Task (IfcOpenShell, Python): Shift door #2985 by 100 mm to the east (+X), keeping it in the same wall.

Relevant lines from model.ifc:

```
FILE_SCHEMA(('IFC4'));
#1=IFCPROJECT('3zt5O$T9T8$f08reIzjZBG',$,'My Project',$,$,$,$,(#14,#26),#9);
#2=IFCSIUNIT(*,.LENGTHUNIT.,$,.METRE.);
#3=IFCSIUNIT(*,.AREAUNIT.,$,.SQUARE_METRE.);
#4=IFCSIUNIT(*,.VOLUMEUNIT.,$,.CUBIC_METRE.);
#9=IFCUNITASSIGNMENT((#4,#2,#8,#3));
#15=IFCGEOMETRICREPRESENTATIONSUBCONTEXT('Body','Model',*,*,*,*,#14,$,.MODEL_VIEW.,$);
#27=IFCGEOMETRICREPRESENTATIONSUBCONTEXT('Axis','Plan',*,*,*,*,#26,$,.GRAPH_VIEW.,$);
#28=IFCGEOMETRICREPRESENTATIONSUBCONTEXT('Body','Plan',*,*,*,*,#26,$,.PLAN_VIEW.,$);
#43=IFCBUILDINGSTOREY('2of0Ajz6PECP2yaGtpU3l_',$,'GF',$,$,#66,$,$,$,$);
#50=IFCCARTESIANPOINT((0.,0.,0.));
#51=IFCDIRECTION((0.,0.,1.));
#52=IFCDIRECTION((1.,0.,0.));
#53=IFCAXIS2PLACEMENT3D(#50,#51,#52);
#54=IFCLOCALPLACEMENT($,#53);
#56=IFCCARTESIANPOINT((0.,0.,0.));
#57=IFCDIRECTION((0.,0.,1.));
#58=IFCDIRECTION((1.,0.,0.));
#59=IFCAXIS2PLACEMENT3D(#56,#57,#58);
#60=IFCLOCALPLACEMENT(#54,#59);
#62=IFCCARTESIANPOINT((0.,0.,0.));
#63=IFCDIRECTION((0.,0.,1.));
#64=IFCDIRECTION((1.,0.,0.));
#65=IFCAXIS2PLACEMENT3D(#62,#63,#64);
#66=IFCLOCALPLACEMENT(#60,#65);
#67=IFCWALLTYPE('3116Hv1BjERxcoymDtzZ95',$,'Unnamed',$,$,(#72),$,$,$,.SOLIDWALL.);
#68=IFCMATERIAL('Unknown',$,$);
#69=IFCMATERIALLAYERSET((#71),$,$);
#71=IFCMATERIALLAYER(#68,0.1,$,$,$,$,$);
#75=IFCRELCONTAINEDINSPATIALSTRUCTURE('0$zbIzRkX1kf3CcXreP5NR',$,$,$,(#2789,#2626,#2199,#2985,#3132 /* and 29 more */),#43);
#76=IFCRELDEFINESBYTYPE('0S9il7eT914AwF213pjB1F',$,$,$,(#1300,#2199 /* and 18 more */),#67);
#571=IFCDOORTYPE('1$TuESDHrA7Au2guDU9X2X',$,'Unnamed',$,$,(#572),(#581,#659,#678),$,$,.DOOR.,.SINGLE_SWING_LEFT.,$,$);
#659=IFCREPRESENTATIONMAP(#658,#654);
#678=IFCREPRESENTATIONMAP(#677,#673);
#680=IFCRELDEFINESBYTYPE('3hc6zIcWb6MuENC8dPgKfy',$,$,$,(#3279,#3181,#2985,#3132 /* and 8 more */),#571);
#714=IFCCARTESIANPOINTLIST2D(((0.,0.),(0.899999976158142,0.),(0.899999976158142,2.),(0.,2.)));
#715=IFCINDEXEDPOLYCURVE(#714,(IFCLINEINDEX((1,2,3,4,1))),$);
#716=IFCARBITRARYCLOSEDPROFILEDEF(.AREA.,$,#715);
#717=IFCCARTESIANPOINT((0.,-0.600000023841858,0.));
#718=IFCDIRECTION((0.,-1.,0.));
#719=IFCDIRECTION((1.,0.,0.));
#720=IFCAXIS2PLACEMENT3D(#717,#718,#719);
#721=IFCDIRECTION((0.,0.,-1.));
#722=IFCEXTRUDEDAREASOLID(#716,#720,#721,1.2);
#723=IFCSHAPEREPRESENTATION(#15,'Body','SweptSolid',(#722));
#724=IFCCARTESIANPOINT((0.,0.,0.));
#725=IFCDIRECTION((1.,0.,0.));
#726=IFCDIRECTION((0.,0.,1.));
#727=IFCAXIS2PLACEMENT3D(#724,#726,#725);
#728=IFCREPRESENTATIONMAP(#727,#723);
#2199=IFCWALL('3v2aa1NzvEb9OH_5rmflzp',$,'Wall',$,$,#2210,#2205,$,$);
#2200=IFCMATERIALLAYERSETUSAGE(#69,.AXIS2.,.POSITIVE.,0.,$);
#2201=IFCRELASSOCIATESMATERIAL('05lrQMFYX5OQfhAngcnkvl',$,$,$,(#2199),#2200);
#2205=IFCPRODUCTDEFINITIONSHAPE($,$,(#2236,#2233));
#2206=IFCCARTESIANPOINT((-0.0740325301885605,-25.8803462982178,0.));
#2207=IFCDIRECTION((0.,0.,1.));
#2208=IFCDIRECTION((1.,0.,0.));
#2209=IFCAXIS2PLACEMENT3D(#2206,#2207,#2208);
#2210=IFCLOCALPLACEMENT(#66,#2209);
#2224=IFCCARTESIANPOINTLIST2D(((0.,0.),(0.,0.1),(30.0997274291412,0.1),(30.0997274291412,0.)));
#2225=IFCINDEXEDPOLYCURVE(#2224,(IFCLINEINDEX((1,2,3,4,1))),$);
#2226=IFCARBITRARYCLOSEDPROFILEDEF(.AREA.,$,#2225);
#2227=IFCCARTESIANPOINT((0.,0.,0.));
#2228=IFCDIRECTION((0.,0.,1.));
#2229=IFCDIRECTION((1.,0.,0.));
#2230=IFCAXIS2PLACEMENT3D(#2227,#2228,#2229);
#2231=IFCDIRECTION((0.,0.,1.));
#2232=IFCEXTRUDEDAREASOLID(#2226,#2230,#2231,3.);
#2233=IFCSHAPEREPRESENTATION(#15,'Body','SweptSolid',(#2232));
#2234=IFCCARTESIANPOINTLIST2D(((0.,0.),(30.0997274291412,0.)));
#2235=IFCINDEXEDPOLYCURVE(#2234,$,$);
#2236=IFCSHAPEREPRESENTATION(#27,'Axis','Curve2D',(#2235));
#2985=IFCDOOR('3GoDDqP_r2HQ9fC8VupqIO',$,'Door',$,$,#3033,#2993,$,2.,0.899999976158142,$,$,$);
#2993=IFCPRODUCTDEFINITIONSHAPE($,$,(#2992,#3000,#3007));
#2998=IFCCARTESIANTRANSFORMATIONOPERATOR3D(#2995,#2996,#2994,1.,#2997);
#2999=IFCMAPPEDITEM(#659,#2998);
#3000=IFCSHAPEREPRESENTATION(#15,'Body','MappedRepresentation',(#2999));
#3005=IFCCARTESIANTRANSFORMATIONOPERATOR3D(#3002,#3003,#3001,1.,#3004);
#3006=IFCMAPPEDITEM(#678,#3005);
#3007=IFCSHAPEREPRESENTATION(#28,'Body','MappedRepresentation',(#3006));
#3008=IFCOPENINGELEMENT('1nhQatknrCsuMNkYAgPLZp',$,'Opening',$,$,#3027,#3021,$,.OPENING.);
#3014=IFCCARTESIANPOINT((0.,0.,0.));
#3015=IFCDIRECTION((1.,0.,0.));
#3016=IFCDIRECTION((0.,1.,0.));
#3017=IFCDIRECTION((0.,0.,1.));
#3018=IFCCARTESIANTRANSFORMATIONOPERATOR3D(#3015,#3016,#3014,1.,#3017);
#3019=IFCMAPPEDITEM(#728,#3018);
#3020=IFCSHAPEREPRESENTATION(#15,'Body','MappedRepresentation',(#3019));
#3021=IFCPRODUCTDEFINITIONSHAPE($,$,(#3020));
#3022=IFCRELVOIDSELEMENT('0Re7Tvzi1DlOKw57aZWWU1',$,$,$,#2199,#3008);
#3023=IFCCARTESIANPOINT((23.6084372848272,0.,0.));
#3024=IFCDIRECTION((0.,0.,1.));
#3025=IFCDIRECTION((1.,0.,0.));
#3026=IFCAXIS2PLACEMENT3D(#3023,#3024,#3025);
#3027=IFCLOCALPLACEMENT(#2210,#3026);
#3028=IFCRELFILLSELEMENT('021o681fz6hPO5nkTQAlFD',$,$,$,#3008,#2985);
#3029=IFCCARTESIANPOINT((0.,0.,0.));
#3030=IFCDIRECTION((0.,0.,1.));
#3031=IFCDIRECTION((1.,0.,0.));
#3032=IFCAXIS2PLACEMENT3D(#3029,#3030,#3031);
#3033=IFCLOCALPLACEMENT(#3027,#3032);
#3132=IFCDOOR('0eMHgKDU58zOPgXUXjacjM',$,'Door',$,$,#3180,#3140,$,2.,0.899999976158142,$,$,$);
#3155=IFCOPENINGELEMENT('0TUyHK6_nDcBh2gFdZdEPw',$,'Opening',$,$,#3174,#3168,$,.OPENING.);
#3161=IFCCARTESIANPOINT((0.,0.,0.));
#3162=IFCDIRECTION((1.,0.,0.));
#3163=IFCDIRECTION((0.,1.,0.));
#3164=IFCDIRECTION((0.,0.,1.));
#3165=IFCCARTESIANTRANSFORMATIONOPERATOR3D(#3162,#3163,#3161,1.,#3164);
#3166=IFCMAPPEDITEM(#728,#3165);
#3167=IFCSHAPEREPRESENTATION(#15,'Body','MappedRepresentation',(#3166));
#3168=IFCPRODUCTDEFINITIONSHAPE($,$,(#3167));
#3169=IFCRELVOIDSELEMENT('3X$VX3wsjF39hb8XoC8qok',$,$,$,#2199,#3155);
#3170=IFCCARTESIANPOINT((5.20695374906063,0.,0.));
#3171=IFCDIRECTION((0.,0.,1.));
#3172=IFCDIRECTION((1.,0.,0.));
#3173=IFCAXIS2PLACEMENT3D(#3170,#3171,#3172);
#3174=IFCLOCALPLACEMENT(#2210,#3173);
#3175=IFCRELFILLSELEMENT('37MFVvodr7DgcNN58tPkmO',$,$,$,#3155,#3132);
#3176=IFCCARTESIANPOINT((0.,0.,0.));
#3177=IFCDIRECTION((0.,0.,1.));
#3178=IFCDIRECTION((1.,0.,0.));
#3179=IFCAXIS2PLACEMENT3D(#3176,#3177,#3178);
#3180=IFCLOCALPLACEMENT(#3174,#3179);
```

```python
import ifcopenshell
import ifcopenshell.api.geometry
import ifcopenshell.util.placement

model = ifcopenshell.open("model.ifc")

door = model.by_guid("3GoDDqP_r2HQ9fC8VupqIO")
opening = door.FillsVoids[0].RelatingOpeningElement
wall = opening.VoidsElements[0].RelatingBuildingElement

wall_matrix = ifcopenshell.util.placement.get_local_placement(wall.ObjectPlacement)
shift = wall_matrix[:3, 0] * 0.1
before = ifcopenshell.util.placement.get_local_placement(door.ObjectPlacement)[:3, 3].copy()

# The door is placed relative to its opening, so it follows when the opening moves.
matrix = ifcopenshell.util.placement.get_local_placement(opening.ObjectPlacement)
matrix[:3, 3] += shift
ifcopenshell.api.geometry.edit_object_placement(
    model, product=opening, matrix=matrix, is_si=False, should_transform_children=True
)

after = ifcopenshell.util.placement.get_local_placement(door.ObjectPlacement)[:3, 3]
print("door moved by", (after - before).round(3) + 0.0)

model.write("model-out.ifc")
```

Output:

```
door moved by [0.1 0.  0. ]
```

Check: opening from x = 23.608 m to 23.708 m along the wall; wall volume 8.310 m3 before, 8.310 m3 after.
